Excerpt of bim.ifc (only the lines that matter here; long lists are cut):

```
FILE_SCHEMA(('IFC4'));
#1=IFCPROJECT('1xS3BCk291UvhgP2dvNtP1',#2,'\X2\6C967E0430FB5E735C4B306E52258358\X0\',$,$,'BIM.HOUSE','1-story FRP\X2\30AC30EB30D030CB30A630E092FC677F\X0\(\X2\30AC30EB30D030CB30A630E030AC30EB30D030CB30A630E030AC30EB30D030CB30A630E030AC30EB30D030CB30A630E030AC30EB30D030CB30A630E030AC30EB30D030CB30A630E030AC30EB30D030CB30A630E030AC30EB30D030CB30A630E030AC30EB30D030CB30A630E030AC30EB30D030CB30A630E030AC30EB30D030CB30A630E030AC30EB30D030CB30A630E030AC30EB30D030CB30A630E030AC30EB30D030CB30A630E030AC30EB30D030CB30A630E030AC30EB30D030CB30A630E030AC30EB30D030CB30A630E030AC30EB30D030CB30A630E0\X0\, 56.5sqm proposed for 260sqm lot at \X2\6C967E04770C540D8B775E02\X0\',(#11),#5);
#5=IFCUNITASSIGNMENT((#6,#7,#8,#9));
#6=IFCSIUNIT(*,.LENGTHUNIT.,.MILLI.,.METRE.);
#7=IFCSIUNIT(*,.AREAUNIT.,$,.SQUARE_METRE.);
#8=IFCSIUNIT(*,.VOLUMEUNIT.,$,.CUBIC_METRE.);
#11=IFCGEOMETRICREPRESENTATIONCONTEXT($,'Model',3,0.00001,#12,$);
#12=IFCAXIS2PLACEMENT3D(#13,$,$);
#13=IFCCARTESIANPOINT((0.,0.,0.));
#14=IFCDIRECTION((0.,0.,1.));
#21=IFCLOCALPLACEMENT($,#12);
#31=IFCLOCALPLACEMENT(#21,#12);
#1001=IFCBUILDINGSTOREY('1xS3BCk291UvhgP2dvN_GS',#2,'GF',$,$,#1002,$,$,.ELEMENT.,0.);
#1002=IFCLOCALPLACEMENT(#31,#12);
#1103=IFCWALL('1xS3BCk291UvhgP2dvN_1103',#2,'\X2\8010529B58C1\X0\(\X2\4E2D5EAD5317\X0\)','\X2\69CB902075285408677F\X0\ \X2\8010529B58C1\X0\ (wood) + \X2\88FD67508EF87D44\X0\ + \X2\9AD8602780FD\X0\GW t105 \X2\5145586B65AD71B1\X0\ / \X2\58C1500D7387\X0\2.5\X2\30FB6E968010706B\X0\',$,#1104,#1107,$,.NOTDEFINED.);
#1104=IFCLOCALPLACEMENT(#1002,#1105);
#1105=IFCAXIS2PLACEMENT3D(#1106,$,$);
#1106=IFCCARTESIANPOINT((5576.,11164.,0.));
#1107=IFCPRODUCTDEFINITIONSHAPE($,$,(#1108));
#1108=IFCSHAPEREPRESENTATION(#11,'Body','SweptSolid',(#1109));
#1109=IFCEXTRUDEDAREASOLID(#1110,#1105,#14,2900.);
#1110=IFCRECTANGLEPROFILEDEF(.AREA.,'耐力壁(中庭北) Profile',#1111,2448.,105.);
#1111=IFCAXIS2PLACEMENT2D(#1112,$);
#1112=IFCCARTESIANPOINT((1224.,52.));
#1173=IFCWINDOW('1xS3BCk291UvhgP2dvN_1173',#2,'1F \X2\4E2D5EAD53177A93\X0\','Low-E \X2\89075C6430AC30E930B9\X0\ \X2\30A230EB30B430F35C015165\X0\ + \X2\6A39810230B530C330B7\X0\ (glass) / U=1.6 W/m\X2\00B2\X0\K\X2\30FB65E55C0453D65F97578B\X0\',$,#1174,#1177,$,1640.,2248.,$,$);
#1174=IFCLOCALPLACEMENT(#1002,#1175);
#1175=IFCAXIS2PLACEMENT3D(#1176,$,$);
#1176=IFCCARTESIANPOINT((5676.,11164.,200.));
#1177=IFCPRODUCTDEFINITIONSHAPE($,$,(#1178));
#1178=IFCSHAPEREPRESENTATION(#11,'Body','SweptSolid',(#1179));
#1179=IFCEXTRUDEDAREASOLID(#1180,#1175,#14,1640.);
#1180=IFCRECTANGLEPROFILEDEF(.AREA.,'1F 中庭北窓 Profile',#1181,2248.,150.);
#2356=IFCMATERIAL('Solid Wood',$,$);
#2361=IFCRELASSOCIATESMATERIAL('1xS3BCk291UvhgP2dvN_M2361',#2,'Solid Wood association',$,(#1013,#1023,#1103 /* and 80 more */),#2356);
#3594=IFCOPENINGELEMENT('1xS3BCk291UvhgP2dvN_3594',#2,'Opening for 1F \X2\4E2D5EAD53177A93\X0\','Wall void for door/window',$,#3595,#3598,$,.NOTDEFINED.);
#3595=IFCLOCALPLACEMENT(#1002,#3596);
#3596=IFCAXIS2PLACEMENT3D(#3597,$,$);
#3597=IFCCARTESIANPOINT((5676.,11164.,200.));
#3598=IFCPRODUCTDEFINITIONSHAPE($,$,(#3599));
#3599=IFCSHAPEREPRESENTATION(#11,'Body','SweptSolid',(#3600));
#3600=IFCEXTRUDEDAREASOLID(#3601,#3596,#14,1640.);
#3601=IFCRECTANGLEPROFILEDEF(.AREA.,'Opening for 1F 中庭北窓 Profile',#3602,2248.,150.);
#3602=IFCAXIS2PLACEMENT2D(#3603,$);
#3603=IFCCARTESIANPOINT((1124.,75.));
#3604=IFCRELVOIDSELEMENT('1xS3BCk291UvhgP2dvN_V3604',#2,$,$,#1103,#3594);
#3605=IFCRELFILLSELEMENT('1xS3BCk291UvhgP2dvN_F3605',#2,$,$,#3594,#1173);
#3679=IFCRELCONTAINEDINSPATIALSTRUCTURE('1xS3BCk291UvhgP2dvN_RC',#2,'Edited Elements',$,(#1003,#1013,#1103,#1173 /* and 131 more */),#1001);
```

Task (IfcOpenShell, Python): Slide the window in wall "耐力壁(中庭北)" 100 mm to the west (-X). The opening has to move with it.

```python
import ifcopenshell
import ifcopenshell.api.geometry
import ifcopenshell.util.placement

model = ifcopenshell.open("bim.ifc")

window = model.by_guid("1xS3BCk291UvhgP2dvN_1173")
opening = window.FillsVoids[0].RelatingOpeningElement
wall = opening.VoidsElements[0].RelatingBuildingElement

wall_matrix = ifcopenshell.util.placement.get_local_placement(wall.ObjectPlacement)
shift = wall_matrix[:3, 0] * -100.0
before = ifcopenshell.util.placement.get_local_placement(window.ObjectPlacement)[:3, 3].copy()

# The window is not placed relative to its opening, so move both.
for product in (opening, window):
    matrix = ifcopenshell.util.placement.get_local_placement(product.ObjectPlacement)
    matrix[:3, 3] += shift
    ifcopenshell.api.geometry.edit_object_placement(model, product=product, matrix=matrix, is_si=False)

after = ifcopenshell.util.placement.get_local_placement(window.ObjectPlacement)[:3, 3]
print("window moved by", (after - before).round(3) + 0.0)

model.write("bim-out.ifc")
```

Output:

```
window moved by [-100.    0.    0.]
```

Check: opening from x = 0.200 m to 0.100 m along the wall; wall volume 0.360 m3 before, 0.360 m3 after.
